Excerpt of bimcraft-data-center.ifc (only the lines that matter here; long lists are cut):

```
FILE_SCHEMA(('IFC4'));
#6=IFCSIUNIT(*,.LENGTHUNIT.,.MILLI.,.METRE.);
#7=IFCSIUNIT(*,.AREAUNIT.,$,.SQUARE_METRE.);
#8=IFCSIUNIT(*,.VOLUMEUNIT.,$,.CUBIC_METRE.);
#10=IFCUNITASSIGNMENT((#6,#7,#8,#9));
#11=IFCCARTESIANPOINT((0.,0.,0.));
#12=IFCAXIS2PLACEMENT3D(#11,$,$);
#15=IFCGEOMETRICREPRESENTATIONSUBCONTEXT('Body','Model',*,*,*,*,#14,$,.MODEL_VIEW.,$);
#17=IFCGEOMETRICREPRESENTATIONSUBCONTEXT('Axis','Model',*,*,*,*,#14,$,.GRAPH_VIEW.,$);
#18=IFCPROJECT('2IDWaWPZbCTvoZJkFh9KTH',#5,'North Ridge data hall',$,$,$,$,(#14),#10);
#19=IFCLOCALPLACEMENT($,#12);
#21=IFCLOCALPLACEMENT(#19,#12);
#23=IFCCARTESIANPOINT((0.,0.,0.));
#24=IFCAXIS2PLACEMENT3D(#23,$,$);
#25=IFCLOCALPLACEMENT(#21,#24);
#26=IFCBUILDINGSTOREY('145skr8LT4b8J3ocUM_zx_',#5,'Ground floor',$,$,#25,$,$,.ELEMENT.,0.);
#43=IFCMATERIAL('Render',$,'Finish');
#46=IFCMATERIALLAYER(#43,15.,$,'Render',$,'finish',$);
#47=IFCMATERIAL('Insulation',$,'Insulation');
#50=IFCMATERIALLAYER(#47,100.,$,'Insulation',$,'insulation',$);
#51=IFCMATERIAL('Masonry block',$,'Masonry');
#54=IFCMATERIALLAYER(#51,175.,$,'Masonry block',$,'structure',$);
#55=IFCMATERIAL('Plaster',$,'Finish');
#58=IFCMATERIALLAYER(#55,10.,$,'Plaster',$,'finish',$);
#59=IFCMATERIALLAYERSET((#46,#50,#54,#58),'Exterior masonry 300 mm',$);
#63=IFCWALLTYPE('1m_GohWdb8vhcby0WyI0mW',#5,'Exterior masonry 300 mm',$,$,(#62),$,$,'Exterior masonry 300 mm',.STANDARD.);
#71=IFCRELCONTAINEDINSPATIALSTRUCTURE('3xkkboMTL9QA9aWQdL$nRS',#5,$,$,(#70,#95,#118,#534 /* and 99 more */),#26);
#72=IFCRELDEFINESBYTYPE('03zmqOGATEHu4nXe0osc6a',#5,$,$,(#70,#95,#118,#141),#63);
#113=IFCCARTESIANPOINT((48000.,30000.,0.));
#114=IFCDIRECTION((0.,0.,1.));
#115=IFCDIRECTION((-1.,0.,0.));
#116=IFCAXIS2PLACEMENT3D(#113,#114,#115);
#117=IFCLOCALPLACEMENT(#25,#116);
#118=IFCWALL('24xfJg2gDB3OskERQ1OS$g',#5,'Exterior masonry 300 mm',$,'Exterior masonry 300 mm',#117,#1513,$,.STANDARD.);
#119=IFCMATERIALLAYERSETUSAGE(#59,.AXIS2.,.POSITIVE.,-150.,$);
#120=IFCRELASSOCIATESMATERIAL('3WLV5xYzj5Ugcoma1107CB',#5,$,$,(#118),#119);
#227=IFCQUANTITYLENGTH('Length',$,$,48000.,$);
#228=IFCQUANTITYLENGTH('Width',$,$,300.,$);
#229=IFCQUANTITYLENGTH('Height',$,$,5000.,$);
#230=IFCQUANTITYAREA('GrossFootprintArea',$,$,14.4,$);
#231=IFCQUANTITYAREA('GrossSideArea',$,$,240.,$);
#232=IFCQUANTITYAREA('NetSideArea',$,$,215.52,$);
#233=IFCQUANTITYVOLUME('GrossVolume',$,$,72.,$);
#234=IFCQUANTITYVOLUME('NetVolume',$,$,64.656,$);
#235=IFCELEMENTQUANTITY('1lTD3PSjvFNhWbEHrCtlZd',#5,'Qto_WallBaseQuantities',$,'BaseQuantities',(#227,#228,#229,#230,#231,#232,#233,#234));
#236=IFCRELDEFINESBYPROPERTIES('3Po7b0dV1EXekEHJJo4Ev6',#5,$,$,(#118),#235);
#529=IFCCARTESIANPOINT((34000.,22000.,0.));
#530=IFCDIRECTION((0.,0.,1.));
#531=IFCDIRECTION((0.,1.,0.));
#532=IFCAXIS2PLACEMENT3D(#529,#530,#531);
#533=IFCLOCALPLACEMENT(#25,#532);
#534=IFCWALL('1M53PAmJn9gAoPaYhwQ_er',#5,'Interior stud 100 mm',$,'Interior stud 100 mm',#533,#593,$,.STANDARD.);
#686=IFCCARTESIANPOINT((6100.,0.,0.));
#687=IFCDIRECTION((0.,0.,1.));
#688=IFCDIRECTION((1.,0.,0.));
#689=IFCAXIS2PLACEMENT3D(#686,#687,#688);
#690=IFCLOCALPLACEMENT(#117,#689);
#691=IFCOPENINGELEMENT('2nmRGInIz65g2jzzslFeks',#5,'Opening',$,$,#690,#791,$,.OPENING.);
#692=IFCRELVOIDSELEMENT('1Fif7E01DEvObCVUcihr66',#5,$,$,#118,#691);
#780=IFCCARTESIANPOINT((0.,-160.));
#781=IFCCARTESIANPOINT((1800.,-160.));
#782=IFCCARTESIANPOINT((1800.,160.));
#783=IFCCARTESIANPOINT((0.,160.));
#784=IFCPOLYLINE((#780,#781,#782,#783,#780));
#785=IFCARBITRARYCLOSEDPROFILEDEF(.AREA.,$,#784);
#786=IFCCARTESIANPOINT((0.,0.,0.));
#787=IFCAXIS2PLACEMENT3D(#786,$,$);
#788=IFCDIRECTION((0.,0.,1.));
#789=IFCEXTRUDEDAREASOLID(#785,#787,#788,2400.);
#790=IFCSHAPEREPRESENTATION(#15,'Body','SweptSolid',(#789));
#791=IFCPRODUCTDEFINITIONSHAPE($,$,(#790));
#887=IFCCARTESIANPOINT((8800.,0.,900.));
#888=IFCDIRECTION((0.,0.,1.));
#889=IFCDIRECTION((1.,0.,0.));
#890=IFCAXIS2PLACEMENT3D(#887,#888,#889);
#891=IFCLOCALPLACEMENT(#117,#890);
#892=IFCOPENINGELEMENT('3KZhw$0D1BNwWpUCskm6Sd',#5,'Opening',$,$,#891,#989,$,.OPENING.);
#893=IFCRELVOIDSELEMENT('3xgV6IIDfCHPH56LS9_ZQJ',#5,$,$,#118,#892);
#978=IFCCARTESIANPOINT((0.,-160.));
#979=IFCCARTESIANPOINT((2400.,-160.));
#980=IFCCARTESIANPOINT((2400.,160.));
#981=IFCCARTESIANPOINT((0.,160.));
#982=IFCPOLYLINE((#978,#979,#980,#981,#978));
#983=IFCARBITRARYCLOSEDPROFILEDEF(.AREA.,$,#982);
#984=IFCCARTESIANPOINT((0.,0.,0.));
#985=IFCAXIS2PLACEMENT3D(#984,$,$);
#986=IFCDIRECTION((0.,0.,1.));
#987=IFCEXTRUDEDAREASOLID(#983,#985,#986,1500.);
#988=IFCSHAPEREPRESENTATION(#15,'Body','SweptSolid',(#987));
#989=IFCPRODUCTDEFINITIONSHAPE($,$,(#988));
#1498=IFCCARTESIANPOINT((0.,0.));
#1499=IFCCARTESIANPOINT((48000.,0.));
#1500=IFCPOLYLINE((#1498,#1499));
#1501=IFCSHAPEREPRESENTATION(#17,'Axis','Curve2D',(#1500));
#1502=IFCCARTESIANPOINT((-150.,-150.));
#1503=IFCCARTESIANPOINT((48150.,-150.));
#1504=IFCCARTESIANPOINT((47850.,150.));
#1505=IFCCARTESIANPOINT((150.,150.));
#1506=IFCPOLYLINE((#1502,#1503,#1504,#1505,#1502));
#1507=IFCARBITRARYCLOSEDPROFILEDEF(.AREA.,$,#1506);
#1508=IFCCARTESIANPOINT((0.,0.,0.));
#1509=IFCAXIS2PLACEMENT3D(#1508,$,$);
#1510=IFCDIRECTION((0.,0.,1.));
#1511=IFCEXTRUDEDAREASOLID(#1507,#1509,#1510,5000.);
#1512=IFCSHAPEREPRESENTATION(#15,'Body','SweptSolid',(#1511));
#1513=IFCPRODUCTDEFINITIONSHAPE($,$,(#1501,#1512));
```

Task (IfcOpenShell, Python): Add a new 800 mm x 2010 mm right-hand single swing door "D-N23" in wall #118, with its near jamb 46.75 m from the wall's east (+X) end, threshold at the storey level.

```python
import numpy as np
import ifcopenshell
import ifcopenshell.api.feature
import ifcopenshell.api.geometry
import ifcopenshell.api.pset
import ifcopenshell.api.root
import ifcopenshell.api.spatial
import ifcopenshell.geom
import ifcopenshell.util.element
import ifcopenshell.util.placement
import ifcopenshell.util.representation
import ifcopenshell.util.shape
import ifcopenshell.util.unit

model = ifcopenshell.open("bimcraft-data-center.ifc")
unit_scale = ifcopenshell.util.unit.calculate_unit_scale(model)
area_scale = ifcopenshell.util.unit.calculate_unit_scale(model, "AREAUNIT")
volume_scale = ifcopenshell.util.unit.calculate_unit_scale(model, "VOLUMEUNIT")
settings = ifcopenshell.geom.settings()


def volume(element):
    """Net volume in cubic metres, openings subtracted."""
    shape = ifcopenshell.geom.create_shape(settings, element)
    return ifcopenshell.util.shape.get_volume(shape.geometry)


wall = model.by_id(118)
storey = ifcopenshell.util.element.get_container(wall, ifc_class="IfcBuildingStorey")
context = ifcopenshell.util.representation.get_context(model, "Model", "Body", "MODEL_VIEW")
before = volume(wall)

width, height, from_end, sill = 0.8, 2.01, 46.75, 0.0  # metres

# The wall runs along its own X axis, and the end named is its -X end.
wall_shape = ifcopenshell.geom.create_shape(settings, wall)
x, y, z = ifcopenshell.util.shape.get_vertices(wall_shape.geometry).T
start = x.min() + from_end
face, thickness = float(y.min()), float(y.max() - y.min())
wall_matrix = ifcopenshell.util.placement.get_local_placement(wall.ObjectPlacement)
level = ifcopenshell.util.placement.get_local_placement(storey.ObjectPlacement)[2, 3]


def in_wall(x, y):
    """Placement at x, y metres in the wall's axes, at sill height."""
    matrix = wall_matrix.copy()
    matrix[:, 3] = wall_matrix @ np.array([x / unit_scale, y / unit_scale, 0.0, 1.0])
    matrix[2, 3] = level + sill / unit_scale
    return matrix


# Opening: a box that overshoots both wall faces by 50 mm.
opening = ifcopenshell.api.root.create_entity(model, ifc_class="IfcOpeningElement", predefined_type="OPENING")
box = ifcopenshell.api.geometry.add_wall_representation(
    model, context=context, length=width, height=height, thickness=thickness + 0.1
)
ifcopenshell.api.geometry.assign_representation(model, product=opening, representation=box)
ifcopenshell.api.geometry.edit_object_placement(model, product=opening, matrix=in_wall(start, face - 0.05), is_si=False)
ifcopenshell.api.feature.add_feature(model, feature=opening, element=wall)

door = ifcopenshell.api.root.create_entity(model, ifc_class="IfcDoor", name="D-N23", predefined_type="DOOR")
door.OverallWidth, door.OverallHeight = width / unit_scale, height / unit_scale
door.OperationType = "SINGLE_SWING_RIGHT"
body = ifcopenshell.api.geometry.add_door_representation(
    model,
    context=context,
    overall_width=door.OverallWidth,
    overall_height=door.OverallHeight,
    operation_type="SINGLE_SWING_RIGHT",
    lining_properties={"LiningDepth": thickness / unit_scale, "ThresholdDepth": thickness / unit_scale},
)
ifcopenshell.api.geometry.assign_representation(model, product=door, representation=body)
ifcopenshell.api.spatial.assign_container(model, products=[door], relating_structure=storey)
ifcopenshell.api.feature.add_filling(model, opening=opening, element=door)

# The lining spans the wall, so the door starts at the wall face.
ifcopenshell.api.geometry.edit_object_placement(model, product=door, matrix=in_wall(start, face), is_si=False)

after = volume(wall)

# Update the wall's stored quantities.
qto = model.by_id(ifcopenshell.util.element.get_pset(wall, "Qto_WallBaseQuantities", should_inherit=False)["id"])
ifcopenshell.api.pset.edit_qto(model, qto=qto, properties={
    "NetSideArea": after / thickness / area_scale,
    "NetVolume": after / volume_scale,
})

print(f"wall volume {before:.3f} -> {after:.3f} m3")

model.write("bimcraft-data-center_updated.ifc")
```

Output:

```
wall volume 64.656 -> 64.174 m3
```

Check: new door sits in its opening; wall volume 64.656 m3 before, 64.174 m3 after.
